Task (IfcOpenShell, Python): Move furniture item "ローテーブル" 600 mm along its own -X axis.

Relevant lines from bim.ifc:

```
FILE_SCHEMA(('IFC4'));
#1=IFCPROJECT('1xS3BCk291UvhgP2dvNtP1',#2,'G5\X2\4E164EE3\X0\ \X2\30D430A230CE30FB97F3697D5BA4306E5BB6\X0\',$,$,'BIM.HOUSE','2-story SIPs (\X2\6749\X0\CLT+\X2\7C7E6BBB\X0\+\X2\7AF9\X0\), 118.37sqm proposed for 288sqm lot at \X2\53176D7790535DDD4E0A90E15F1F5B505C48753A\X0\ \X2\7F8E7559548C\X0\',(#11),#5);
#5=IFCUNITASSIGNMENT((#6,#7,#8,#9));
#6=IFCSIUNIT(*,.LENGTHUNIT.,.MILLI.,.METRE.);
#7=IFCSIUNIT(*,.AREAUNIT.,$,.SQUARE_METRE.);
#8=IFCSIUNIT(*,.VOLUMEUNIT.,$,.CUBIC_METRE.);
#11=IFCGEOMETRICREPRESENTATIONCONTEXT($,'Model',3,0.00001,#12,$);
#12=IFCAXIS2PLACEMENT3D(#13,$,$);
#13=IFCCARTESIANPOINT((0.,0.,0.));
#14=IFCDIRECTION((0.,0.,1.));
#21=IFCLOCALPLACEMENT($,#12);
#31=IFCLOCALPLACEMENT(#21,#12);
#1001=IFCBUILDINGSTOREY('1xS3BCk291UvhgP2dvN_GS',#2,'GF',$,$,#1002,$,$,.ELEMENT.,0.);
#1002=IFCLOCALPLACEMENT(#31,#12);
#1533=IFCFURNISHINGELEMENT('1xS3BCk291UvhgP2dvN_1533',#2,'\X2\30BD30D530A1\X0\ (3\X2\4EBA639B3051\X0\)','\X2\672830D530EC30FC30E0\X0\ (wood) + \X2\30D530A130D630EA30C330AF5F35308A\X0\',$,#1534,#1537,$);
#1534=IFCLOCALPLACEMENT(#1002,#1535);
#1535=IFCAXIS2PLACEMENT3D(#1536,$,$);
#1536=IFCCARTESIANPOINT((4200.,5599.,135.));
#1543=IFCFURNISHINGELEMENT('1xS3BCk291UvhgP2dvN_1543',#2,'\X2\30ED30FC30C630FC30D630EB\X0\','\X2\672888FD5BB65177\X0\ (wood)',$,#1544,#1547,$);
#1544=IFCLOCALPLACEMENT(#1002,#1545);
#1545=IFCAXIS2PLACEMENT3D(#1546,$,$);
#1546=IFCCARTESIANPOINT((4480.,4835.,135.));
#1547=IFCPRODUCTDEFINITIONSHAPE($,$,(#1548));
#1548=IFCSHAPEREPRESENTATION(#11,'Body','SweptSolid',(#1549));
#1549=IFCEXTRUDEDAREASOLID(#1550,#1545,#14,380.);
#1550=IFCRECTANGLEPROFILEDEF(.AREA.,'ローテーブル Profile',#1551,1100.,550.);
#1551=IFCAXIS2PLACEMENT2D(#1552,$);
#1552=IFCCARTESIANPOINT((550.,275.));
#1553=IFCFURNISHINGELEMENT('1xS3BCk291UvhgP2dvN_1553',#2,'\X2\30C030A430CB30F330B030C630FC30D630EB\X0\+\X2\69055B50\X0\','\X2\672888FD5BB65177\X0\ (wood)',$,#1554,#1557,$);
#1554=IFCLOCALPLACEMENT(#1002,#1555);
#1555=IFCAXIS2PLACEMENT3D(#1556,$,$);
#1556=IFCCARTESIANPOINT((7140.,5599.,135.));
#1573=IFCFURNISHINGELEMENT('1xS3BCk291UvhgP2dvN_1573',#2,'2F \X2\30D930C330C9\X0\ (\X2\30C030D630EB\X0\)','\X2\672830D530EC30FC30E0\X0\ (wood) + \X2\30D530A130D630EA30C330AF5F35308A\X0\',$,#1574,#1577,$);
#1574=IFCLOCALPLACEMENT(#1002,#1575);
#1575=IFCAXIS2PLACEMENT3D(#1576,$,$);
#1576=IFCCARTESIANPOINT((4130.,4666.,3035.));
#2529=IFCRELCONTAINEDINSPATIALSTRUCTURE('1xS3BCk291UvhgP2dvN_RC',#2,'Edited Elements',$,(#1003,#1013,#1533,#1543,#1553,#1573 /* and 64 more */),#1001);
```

```python
import ifcopenshell
import ifcopenshell.api.geometry
import ifcopenshell.util.placement
import ifcopenshell.util.unit

model = ifcopenshell.open("bim.ifc")
unit_scale = ifcopenshell.util.unit.calculate_unit_scale(model)

item = model.by_guid("1xS3BCk291UvhgP2dvN_1543")
matrix = ifcopenshell.util.placement.get_local_placement(item.ObjectPlacement)
matrix[:3, 3] -= matrix[:3, 0] * 0.6 / unit_scale
ifcopenshell.api.geometry.edit_object_placement(model, product=item, matrix=matrix, is_si=False)

print(ifcopenshell.util.placement.get_local_placement(item.ObjectPlacement).round(3) + 0.0)

model.write("bim_updated.ifc")
```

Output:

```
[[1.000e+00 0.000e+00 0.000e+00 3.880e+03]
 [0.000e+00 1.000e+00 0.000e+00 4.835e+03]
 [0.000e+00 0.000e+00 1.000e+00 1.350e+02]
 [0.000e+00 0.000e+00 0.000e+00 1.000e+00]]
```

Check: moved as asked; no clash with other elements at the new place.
